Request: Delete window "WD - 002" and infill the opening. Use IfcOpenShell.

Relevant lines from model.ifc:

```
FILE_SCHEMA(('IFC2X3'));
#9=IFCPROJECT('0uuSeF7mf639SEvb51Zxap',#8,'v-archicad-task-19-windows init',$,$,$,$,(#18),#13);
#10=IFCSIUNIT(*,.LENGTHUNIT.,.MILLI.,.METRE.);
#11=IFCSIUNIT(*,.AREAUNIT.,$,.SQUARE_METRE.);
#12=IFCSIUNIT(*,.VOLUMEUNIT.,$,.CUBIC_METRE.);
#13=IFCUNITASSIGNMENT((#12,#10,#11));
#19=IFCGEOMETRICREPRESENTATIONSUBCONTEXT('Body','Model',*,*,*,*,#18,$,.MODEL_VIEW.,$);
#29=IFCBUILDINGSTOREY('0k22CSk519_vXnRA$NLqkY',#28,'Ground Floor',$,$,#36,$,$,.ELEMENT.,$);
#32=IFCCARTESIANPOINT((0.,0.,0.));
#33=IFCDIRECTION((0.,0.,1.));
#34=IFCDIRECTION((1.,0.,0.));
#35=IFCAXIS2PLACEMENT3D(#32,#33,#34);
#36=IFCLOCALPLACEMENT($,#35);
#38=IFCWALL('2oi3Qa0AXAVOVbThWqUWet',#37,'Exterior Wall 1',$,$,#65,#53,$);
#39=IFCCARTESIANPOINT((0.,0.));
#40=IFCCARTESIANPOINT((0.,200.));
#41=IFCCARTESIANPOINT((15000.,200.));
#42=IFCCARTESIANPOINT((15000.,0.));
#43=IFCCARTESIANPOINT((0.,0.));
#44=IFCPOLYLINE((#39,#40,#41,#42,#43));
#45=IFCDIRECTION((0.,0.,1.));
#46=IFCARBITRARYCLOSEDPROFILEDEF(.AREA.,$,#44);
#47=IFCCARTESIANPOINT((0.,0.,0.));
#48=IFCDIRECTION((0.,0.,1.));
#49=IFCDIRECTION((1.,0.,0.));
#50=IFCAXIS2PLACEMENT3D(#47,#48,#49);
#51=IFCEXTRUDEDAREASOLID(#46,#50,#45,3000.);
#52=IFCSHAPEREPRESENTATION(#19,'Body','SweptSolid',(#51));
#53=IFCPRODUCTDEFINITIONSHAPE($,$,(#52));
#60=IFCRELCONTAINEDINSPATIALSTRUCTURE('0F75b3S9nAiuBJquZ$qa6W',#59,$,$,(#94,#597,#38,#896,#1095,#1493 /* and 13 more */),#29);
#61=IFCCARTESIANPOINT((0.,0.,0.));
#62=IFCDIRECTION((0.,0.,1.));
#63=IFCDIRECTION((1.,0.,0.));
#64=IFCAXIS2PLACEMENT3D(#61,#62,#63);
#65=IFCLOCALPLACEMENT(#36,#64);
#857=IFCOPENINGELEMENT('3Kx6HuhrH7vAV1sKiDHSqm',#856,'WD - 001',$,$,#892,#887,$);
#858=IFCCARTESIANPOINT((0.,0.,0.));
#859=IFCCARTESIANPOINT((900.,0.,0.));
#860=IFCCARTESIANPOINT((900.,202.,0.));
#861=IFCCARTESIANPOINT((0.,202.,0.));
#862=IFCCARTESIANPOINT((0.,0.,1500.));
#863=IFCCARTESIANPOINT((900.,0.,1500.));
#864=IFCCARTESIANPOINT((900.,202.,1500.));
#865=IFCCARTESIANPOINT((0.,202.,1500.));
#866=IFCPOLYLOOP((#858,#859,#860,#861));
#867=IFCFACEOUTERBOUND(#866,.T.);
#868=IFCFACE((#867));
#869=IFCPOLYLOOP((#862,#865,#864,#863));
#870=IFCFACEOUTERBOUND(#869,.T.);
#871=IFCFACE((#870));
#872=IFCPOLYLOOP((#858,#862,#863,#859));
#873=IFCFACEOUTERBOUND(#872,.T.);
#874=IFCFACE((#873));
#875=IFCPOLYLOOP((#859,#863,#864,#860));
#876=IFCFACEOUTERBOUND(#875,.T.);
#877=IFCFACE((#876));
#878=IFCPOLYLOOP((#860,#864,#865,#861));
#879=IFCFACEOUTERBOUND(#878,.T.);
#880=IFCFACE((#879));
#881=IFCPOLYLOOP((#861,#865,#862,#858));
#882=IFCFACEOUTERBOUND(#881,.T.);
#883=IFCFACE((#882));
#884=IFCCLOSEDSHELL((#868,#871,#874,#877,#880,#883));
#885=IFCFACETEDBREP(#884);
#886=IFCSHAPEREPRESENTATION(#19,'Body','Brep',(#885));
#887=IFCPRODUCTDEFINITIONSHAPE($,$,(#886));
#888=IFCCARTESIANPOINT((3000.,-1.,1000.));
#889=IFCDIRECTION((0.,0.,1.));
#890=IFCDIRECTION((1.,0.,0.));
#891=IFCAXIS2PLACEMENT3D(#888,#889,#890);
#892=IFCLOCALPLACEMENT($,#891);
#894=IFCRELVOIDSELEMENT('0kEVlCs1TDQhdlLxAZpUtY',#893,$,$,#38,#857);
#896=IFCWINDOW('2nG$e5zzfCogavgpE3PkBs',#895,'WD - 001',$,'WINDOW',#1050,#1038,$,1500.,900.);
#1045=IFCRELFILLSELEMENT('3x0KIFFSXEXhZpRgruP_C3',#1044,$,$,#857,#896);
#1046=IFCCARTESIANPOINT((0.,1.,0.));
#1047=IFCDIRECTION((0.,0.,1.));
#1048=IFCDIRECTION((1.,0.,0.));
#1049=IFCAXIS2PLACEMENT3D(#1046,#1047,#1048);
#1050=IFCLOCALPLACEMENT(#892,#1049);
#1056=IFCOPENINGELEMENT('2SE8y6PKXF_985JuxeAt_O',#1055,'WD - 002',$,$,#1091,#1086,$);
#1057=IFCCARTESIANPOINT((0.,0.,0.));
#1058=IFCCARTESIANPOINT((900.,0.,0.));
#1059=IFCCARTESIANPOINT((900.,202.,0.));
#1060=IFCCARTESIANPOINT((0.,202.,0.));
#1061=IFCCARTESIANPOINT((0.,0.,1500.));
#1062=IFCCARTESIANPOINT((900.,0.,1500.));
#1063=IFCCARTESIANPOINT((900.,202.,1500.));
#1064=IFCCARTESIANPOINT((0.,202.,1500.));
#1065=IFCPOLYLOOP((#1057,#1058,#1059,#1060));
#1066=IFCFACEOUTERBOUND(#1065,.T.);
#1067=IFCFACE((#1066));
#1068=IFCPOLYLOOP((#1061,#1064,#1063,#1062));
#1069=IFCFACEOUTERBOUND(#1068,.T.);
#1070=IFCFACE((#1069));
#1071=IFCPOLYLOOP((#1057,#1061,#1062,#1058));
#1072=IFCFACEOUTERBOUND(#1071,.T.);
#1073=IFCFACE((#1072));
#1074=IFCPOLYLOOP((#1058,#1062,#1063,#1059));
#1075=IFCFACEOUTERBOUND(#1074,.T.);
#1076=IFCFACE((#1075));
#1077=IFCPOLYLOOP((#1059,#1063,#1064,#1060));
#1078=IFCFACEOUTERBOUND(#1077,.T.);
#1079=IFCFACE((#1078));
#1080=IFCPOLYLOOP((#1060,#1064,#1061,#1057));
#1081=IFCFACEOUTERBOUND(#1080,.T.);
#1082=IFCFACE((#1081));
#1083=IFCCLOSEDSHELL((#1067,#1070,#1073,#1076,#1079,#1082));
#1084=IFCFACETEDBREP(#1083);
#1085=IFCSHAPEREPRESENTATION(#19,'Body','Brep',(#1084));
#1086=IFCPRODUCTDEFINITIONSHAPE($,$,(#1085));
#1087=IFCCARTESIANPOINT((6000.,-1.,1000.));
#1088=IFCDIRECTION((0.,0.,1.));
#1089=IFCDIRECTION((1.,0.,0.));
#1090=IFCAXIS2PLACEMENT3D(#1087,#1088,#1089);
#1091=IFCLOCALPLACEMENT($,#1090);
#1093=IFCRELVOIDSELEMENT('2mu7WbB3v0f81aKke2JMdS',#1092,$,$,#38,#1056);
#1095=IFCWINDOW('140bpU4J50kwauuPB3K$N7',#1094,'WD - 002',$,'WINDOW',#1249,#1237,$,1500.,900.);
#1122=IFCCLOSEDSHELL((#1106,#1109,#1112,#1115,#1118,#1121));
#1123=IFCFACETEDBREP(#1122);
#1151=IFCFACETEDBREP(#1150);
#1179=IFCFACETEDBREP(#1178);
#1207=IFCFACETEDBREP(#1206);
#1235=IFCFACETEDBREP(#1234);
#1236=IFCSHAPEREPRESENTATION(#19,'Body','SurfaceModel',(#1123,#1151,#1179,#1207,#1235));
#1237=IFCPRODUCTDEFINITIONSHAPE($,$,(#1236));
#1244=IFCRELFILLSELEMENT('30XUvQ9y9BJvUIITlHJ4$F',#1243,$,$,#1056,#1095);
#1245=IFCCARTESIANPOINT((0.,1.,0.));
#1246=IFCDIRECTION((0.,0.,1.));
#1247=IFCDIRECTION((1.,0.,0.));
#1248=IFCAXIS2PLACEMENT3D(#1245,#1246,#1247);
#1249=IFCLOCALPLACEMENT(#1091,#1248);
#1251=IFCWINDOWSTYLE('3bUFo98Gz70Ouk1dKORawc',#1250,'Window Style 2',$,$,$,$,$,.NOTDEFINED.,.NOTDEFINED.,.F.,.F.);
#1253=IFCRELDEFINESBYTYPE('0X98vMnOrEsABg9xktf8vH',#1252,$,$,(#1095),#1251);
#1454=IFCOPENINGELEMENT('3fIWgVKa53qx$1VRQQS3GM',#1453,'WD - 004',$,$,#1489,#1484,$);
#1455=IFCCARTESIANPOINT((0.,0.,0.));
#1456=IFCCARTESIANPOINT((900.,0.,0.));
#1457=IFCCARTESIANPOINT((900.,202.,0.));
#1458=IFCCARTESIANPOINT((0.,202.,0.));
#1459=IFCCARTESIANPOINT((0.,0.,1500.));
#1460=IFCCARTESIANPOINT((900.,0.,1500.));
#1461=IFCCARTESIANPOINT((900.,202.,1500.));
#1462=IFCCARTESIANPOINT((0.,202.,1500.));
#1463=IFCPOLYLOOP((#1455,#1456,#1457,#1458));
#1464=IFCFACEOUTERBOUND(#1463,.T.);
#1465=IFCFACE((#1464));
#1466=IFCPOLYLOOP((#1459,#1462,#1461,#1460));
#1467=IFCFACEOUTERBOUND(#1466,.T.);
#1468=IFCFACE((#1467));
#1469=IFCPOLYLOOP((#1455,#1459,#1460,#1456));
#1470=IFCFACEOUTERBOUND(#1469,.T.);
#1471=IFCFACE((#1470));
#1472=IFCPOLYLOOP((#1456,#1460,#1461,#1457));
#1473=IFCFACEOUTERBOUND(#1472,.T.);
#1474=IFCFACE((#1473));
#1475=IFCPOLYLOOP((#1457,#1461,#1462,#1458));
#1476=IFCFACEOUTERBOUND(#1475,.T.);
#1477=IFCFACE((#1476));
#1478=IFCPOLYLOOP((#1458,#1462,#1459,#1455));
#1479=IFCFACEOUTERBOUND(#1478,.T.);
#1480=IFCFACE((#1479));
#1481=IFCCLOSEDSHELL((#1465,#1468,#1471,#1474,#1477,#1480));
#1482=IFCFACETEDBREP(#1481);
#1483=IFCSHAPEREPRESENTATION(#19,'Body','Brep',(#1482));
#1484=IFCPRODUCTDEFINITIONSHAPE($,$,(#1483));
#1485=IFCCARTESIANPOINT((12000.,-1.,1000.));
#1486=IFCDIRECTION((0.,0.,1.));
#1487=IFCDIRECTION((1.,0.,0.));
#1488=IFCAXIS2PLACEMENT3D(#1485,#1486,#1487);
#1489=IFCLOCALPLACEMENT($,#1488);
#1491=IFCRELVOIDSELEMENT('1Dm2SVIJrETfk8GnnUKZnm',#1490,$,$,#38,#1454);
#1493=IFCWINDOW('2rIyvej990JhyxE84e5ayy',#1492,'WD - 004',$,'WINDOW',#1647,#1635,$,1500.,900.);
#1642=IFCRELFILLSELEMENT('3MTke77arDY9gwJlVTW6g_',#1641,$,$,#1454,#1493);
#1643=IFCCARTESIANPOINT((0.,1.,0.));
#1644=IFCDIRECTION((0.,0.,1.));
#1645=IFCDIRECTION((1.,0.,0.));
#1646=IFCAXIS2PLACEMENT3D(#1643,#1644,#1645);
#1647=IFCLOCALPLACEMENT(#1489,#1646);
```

```python
import ifcopenshell
import ifcopenshell.api.feature
import ifcopenshell.api.root
import ifcopenshell.geom
import ifcopenshell.util.shape

model = ifcopenshell.open("model.ifc")
settings = ifcopenshell.geom.settings()


def volume(element):
    """Net volume in cubic metres, openings subtracted."""
    shape = ifcopenshell.geom.create_shape(settings, element)
    return ifcopenshell.util.shape.get_volume(shape.geometry)


window = model.by_guid("140bpU4J50kwauuPB3K$N7")
opening = window.FillsVoids[0].RelatingOpeningElement
wall = opening.VoidsElements[0].RelatingBuildingElement
before = volume(wall)

ifcopenshell.api.root.remove_product(model, product=window)
ifcopenshell.api.feature.remove_feature(model, feature=opening)

after = volume(wall)

print(f"wall volume {before:.3f} -> {after:.3f} m3")

model.write("model_rev.ifc")
```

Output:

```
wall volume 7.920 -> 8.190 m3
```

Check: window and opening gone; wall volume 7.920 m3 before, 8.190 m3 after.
